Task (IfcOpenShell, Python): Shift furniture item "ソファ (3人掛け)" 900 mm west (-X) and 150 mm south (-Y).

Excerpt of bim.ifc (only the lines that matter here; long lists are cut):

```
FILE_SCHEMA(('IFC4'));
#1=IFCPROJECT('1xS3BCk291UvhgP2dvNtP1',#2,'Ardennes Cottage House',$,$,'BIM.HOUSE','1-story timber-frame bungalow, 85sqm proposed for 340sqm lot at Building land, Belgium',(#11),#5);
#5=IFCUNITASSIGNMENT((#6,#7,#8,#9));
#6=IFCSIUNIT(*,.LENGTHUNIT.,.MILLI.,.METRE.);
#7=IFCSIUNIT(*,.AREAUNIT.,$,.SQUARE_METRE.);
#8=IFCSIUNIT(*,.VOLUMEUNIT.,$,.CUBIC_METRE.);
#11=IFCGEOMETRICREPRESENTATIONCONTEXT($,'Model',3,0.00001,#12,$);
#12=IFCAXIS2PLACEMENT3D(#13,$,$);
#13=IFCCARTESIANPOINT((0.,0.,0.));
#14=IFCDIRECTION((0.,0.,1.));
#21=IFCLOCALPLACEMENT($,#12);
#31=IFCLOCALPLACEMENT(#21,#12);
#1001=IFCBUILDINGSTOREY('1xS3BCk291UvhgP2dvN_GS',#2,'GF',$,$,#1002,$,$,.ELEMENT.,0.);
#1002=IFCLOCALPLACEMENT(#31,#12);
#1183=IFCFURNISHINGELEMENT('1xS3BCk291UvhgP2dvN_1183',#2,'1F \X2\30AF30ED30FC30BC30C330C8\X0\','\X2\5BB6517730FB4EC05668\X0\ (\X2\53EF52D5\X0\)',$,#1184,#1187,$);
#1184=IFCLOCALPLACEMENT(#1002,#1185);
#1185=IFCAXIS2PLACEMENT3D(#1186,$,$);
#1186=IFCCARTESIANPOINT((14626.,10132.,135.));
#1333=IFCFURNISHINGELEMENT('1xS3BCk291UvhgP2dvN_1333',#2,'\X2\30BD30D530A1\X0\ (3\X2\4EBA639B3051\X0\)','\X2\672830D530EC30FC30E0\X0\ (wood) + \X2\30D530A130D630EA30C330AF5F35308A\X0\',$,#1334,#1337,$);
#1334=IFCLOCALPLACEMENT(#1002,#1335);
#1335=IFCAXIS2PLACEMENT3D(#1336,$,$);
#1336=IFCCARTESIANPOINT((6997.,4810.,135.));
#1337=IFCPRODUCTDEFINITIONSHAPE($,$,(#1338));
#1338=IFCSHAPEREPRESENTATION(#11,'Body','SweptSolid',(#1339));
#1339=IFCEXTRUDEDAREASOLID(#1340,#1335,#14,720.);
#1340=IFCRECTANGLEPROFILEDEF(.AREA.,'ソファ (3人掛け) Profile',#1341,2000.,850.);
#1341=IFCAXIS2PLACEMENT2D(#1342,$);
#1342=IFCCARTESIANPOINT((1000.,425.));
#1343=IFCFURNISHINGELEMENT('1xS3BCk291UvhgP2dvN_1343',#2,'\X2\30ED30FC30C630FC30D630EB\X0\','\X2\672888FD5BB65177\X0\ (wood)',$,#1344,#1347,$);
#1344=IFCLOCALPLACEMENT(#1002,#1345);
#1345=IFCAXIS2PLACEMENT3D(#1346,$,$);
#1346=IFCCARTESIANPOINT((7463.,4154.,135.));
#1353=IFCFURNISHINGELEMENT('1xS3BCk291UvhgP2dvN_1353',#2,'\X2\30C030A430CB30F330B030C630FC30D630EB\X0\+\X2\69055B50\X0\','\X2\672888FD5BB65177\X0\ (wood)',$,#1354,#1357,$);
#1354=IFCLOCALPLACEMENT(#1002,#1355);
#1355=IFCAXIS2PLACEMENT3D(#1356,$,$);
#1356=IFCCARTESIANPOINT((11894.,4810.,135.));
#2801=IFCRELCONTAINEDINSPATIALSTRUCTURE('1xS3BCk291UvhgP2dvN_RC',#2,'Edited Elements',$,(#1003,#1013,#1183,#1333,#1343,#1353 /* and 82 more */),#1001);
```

```python
import ifcopenshell
import ifcopenshell.api.geometry
import ifcopenshell.util.placement
import ifcopenshell.util.unit

model = ifcopenshell.open("bim.ifc")
unit_scale = ifcopenshell.util.unit.calculate_unit_scale(model)

item = model.by_guid("1xS3BCk291UvhgP2dvN_1333")
matrix = ifcopenshell.util.placement.get_local_placement(item.ObjectPlacement)
matrix[0, 3] -= 0.9 / unit_scale
matrix[1, 3] -= 0.15 / unit_scale
ifcopenshell.api.geometry.edit_object_placement(model, product=item, matrix=matrix, is_si=False)

print(ifcopenshell.util.placement.get_local_placement(item.ObjectPlacement).round(3) + 0.0)

model.write("bim_updated.ifc")
```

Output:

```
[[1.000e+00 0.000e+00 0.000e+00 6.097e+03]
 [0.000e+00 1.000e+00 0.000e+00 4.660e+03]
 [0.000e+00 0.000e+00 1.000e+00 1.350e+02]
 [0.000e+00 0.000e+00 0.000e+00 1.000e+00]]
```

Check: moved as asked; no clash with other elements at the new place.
